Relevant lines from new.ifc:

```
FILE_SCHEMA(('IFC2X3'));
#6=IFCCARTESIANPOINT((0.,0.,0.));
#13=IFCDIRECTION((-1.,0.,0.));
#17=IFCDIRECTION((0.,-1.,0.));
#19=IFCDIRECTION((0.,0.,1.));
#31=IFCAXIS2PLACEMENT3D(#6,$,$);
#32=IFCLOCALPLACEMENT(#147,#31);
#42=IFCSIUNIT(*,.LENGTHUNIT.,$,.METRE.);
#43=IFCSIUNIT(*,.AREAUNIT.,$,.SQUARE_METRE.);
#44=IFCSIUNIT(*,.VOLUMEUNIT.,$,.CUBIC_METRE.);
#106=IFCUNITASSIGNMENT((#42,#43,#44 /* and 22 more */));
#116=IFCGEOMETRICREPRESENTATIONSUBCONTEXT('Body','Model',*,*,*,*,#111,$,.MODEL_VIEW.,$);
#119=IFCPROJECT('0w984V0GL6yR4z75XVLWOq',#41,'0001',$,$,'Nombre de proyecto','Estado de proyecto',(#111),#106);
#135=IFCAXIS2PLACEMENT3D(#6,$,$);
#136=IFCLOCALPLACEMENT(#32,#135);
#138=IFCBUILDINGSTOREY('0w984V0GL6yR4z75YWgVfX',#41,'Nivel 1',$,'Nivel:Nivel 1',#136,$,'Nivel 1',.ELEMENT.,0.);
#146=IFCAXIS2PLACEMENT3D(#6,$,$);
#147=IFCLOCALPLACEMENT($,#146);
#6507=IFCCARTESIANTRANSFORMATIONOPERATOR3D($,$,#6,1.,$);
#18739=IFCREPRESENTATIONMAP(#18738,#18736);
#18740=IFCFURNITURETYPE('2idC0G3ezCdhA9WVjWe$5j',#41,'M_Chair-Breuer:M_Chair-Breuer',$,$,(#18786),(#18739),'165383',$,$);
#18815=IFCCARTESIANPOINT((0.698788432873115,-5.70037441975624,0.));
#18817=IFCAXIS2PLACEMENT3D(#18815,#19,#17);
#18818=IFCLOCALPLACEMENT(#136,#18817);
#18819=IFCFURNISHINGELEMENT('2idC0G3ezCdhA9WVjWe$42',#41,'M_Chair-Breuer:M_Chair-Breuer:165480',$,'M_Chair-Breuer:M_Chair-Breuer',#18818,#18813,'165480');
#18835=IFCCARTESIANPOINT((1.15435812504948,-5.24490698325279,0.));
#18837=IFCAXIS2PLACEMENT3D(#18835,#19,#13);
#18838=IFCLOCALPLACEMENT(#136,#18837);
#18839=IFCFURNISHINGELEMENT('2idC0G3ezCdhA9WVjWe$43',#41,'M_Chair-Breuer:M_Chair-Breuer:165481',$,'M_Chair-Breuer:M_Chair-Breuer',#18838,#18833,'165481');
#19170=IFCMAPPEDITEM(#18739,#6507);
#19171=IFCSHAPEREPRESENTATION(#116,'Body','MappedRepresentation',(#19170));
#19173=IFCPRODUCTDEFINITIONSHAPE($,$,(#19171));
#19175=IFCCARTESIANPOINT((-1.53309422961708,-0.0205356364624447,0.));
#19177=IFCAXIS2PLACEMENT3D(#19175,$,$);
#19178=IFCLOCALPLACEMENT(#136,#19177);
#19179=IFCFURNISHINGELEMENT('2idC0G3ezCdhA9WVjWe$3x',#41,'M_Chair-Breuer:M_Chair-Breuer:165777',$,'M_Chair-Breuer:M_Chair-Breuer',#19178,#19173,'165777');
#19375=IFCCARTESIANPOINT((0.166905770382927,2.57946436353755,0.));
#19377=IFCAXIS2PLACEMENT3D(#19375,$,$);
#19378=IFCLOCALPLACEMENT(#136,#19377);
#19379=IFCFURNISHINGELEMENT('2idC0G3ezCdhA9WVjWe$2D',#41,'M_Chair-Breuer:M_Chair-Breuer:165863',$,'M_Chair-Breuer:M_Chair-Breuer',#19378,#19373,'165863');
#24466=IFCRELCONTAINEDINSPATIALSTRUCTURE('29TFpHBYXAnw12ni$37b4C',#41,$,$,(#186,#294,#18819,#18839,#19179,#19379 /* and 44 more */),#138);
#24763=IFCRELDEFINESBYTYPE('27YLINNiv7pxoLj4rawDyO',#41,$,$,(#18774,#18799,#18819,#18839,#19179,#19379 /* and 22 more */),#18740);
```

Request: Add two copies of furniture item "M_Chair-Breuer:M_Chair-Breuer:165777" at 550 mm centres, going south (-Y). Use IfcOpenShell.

```python
import numpy as np
import ifcopenshell
import ifcopenshell.api.geometry
import ifcopenshell.api.root
import ifcopenshell.util.element
import ifcopenshell.util.placement

model = ifcopenshell.open("new.ifc")


def reuse_history(source, copy):
    """copy_class also copies each property set's owner history, people and application; keep the originals."""
    for rel in copy.IsDefinedBy:
        if rel.is_a("IfcRelDefinesByProperties") and (history := rel.RelatingPropertyDefinition.OwnerHistory):
            rel.RelatingPropertyDefinition.OwnerHistory = source.OwnerHistory
            ifcopenshell.util.element.remove_deep2(model, history)


source = model.by_id(19179)
base = ifcopenshell.util.placement.get_local_placement(source.ObjectPlacement)
step = np.array([0.0, -1.0, 0.0]) * 0.55

for i in range(1, 3):
    copy = ifcopenshell.api.root.copy_class(model, product=source)
    copy.Representation = ifcopenshell.util.element.copy_deep(
        model, source.Representation, exclude=["IfcGeometricRepresentationContext", "IfcRepresentationMap"]
    )
    copy.Name = "M_Chair-Breuer:M_Chair-Breuer"
    copy.Tag = None
    reuse_history(source, copy)
    matrix = base.copy()
    matrix[:3, 3] += i * step
    print("added at", matrix[:3, 3].round(3) + 0.0)
    ifcopenshell.api.geometry.edit_object_placement(model, product=copy, matrix=matrix, is_si=False)

model.write("new_v2.ifc")
```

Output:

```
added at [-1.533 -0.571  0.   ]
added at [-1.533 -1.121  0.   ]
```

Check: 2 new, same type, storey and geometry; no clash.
